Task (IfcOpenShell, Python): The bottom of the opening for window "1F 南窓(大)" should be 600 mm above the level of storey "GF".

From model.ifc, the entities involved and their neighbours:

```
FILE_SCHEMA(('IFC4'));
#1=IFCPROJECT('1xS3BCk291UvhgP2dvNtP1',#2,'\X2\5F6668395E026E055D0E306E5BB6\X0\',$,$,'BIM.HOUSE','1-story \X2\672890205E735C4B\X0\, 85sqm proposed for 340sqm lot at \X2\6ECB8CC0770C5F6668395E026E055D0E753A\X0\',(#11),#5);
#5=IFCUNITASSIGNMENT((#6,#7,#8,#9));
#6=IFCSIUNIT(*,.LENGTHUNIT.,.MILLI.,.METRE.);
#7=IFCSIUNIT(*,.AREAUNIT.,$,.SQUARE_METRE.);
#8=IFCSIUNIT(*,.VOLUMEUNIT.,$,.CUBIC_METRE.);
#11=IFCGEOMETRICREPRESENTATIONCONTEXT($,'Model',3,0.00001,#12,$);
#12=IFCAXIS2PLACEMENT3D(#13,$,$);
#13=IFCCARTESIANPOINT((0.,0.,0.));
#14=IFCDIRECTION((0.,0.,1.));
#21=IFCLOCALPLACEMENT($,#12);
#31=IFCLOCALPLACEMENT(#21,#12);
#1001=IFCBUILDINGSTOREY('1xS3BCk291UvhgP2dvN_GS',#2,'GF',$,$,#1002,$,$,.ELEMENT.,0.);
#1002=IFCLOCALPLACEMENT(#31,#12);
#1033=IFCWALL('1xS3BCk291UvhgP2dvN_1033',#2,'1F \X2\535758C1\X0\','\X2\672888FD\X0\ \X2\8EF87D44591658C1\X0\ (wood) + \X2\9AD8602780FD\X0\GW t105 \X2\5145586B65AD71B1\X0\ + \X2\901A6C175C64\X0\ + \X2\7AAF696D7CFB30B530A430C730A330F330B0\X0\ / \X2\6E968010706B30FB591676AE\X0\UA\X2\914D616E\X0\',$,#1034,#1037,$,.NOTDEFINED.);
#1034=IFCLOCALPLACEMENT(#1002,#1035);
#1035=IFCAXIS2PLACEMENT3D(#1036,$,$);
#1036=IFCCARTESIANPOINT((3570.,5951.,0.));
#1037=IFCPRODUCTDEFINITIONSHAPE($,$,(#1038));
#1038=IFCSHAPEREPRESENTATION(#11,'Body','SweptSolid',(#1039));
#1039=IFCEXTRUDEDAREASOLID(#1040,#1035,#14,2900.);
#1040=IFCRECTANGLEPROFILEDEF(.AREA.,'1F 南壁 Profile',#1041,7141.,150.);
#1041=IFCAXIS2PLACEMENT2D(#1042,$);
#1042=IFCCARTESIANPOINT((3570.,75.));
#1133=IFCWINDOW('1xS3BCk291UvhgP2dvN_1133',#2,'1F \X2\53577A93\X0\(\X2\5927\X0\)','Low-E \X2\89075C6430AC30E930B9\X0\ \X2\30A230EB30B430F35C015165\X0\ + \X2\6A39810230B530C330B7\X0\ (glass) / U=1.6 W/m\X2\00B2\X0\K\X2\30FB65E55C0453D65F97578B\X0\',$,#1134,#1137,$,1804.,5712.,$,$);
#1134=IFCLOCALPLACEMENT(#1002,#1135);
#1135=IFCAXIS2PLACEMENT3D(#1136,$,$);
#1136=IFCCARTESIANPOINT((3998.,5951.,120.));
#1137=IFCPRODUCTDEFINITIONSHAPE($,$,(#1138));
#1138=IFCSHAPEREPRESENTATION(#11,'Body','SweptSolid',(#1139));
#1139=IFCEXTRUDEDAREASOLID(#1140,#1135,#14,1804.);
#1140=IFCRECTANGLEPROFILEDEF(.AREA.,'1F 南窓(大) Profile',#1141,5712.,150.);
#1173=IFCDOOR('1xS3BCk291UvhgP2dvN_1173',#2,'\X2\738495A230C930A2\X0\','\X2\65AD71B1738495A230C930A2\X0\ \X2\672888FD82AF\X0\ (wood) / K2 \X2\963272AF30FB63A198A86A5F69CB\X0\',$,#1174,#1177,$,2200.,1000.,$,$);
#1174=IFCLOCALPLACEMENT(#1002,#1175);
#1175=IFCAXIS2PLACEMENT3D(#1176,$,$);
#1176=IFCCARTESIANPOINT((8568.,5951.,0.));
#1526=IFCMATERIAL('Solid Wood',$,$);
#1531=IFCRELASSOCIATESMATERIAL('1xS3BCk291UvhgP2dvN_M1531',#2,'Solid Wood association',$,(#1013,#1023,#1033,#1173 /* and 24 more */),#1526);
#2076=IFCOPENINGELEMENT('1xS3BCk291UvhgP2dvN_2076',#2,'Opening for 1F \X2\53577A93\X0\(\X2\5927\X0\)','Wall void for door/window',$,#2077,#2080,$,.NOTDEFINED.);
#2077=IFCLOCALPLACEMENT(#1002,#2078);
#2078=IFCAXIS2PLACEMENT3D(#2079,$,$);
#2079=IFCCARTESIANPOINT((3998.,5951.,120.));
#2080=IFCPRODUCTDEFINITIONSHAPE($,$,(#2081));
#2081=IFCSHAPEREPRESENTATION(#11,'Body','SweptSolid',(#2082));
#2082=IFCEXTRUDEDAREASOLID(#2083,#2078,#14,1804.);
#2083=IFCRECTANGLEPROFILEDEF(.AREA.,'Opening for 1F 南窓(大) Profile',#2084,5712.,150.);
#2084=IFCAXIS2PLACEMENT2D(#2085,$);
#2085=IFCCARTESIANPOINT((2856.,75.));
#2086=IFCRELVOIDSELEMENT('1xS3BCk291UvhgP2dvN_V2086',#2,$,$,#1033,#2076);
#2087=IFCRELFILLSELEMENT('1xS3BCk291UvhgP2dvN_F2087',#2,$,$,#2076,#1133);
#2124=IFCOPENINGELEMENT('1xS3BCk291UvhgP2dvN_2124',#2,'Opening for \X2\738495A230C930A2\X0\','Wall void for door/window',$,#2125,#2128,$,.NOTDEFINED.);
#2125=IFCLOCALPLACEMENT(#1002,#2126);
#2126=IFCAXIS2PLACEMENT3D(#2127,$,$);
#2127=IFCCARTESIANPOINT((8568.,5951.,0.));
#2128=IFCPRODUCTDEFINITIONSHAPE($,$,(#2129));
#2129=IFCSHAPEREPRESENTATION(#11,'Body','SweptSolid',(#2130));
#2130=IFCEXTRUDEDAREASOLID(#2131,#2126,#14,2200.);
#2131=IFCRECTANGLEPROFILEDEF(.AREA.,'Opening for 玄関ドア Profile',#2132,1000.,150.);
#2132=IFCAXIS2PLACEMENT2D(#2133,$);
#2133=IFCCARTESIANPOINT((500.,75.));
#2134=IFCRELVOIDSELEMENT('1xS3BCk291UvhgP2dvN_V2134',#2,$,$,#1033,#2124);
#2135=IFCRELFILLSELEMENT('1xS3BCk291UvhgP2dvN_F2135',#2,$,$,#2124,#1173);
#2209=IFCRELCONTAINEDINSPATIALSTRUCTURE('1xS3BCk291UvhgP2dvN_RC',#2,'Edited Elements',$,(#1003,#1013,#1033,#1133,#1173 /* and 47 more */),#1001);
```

```python
import numpy as np
import ifcopenshell
import ifcopenshell.api.geometry
import ifcopenshell.geom
import ifcopenshell.util.element
import ifcopenshell.util.placement
import ifcopenshell.util.shape
import ifcopenshell.util.unit

model = ifcopenshell.open("model.ifc")
unit_scale = ifcopenshell.util.unit.calculate_unit_scale(model)

window = model.by_guid("1xS3BCk291UvhgP2dvN_1133")
opening = window.FillsVoids[0].RelatingOpeningElement
storey = ifcopenshell.util.element.get_container(window, ifc_class="IfcBuildingStorey")
level = ifcopenshell.util.placement.get_local_placement(storey.ObjectPlacement)[2, 3]

# The opening's origin need not be at the sill, so measure its lowest point.
shape = ifcopenshell.geom.create_shape(ifcopenshell.geom.settings(), opening)
bottom = ifcopenshell.util.shape.get_shape_bottom_elevation(shape, shape.geometry) / unit_scale
dz = level + 0.6 / unit_scale - bottom

shift = np.array([0.0, 0.0, dz])
# The window is not placed relative to its opening, so move both.
for product in (opening, window):
    matrix = ifcopenshell.util.placement.get_local_placement(product.ObjectPlacement)
    matrix[:3, 3] += shift
    ifcopenshell.api.geometry.edit_object_placement(model, product=product, matrix=matrix, is_si=False)

print(f"moved by {dz * unit_scale:+.3f} m")

model.write("model-out.ifc")
```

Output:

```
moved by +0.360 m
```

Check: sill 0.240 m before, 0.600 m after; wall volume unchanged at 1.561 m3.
